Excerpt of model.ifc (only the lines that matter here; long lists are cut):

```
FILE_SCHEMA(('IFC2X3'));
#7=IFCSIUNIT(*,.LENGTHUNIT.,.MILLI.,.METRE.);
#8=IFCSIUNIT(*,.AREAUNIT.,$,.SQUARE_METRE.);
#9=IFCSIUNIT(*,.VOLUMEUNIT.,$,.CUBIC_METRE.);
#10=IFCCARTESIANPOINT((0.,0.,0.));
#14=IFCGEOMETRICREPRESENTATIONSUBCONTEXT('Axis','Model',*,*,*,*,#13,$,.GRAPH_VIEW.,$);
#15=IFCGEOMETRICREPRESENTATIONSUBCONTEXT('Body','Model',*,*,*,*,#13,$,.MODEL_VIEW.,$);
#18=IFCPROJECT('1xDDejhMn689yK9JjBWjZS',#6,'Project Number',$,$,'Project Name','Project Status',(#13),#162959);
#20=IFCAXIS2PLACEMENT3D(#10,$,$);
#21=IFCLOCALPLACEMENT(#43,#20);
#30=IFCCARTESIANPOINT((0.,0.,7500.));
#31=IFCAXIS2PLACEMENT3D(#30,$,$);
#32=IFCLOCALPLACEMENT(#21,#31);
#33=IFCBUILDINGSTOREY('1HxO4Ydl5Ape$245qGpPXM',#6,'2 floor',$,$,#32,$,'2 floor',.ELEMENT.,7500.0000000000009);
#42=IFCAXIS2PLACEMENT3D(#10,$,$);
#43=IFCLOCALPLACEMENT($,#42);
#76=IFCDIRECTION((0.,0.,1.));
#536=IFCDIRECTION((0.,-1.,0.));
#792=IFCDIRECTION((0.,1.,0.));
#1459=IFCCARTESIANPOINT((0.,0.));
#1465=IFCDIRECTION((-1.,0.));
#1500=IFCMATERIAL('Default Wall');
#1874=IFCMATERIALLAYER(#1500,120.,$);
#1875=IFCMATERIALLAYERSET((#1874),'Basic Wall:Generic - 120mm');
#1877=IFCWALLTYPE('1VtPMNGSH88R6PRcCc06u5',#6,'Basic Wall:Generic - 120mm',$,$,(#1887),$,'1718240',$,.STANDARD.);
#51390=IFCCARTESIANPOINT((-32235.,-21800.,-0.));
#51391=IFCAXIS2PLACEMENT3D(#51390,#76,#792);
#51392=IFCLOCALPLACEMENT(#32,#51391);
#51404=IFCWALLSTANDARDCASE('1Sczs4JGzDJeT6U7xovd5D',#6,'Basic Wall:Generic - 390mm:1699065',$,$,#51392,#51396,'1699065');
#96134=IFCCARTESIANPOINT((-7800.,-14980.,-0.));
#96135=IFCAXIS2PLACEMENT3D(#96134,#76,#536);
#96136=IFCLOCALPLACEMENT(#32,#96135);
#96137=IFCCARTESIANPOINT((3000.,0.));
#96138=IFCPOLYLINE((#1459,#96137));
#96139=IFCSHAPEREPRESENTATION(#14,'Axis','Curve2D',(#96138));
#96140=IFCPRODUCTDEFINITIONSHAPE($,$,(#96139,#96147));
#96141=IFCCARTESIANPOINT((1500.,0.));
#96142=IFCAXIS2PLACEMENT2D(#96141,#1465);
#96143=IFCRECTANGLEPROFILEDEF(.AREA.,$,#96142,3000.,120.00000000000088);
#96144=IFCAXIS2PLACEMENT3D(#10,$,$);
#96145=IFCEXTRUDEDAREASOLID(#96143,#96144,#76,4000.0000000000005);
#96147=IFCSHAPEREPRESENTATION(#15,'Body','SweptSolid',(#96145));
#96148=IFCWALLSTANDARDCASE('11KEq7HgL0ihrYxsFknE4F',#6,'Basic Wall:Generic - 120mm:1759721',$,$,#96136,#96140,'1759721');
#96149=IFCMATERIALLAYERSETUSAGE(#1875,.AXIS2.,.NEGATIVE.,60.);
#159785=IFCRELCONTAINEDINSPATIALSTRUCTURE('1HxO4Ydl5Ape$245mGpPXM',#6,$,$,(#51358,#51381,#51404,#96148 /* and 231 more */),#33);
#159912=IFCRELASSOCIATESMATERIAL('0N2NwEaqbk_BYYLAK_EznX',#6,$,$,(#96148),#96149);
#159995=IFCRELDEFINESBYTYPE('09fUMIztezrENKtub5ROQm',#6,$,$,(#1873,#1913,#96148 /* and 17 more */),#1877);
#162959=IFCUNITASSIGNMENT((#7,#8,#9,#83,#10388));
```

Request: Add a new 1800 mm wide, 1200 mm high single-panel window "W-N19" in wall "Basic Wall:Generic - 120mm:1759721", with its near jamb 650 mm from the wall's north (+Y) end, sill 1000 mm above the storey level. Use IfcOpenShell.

```python
import numpy as np
import ifcopenshell
import ifcopenshell.api.feature
import ifcopenshell.api.geometry
import ifcopenshell.api.root
import ifcopenshell.api.spatial
import ifcopenshell.api.type
import ifcopenshell.geom
import ifcopenshell.util.element
import ifcopenshell.util.placement
import ifcopenshell.util.representation
import ifcopenshell.util.shape
import ifcopenshell.util.unit

model = ifcopenshell.open("model.ifc")
unit_scale = ifcopenshell.util.unit.calculate_unit_scale(model)
settings = ifcopenshell.geom.settings()


def volume(element):
    """Net volume in cubic metres, openings subtracted."""
    shape = ifcopenshell.geom.create_shape(settings, element)
    return ifcopenshell.util.shape.get_volume(shape.geometry)


wall = model.by_id(96148)
storey = ifcopenshell.util.element.get_container(wall, ifc_class="IfcBuildingStorey")
context = ifcopenshell.util.representation.get_context(model, "Model", "Body", "MODEL_VIEW")
before = volume(wall)

width, height, from_end, sill = 1.8, 1.2, 0.65, 1  # metres

# The wall runs along its own X axis, and the end named is its -X end.
wall_shape = ifcopenshell.geom.create_shape(settings, wall)
x, y, z = ifcopenshell.util.shape.get_vertices(wall_shape.geometry).T
start = x.min() + from_end
face, thickness = float(y.min()), float(y.max() - y.min())
wall_matrix = ifcopenshell.util.placement.get_local_placement(wall.ObjectPlacement)
level = ifcopenshell.util.placement.get_local_placement(storey.ObjectPlacement)[2, 3]


def in_wall(x, y):
    """Placement at x, y metres in the wall's axes, at sill height."""
    matrix = wall_matrix.copy()
    matrix[:, 3] = wall_matrix @ np.array([x / unit_scale, y / unit_scale, 0.0, 1.0])
    matrix[2, 3] = level + sill / unit_scale
    return matrix


# Opening: a box that overshoots both wall faces by 50 mm.
opening = ifcopenshell.api.root.create_entity(model, ifc_class="IfcOpeningElement")
box = ifcopenshell.api.geometry.add_wall_representation(
    model, context=context, length=width, height=height, thickness=thickness + 0.1
)
ifcopenshell.api.geometry.assign_representation(model, product=opening, representation=box)
ifcopenshell.api.geometry.edit_object_placement(model, product=opening, matrix=in_wall(start, face - 0.05), is_si=False)
ifcopenshell.api.feature.add_feature(model, feature=opening, element=wall)

window = ifcopenshell.api.root.create_entity(model, ifc_class="IfcWindow", name="W-N19")
window.OverallWidth, window.OverallHeight = width / unit_scale, height / unit_scale
body = ifcopenshell.api.geometry.add_window_representation(
    model,
    context=context,
    overall_width=window.OverallWidth,
    overall_height=window.OverallHeight,
    partition_type="SINGLE_PANEL",
)
ifcopenshell.api.geometry.assign_representation(model, product=window, representation=body)
ifcopenshell.api.spatial.assign_container(model, products=[window], relating_structure=storey)
fills = ifcopenshell.api.feature.add_filling(model, opening=opening, element=window)
fills.OwnerHistory = window.OwnerHistory  # required in IFC2X3

# IFC2X3 keeps the operation on the window style.
style = ifcopenshell.api.root.create_entity(model, ifc_class="IfcWindowStyle", name="W-N19")
style.OperationType, style.ConstructionType = "SINGLE_PANEL", "NOTDEFINED"
style.ParameterTakesPrecedence = style.Sizeable = False
ifcopenshell.api.type.assign_type(model, related_objects=[window], relating_type=style)

# Centre the window in the wall's thickness.
ifcopenshell.api.geometry.edit_object_placement(model, product=window, matrix=in_wall(start, face), is_si=False)
window_shape = ifcopenshell.geom.create_shape(settings, window)
depth = ifcopenshell.util.shape.get_vertices(window_shape.geometry)[:, 1]
offset = face + thickness / 2 - (depth.min() + depth.max()) / 2
ifcopenshell.api.geometry.edit_object_placement(model, product=window, matrix=in_wall(start, offset), is_si=False)

after = volume(wall)

print(f"wall volume {before:.3f} -> {after:.3f} m3")

model.write("model_rev.ifc")
```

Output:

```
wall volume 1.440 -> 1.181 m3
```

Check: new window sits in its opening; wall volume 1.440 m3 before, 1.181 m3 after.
